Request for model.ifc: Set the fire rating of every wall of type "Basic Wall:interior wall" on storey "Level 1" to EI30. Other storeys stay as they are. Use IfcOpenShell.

First a look at what the model holds.

```python
import ifcopenshell
import ifcopenshell.util.element

model = ifcopenshell.open("model.ifc")
print(model.schema)
storey = next(s for s in model.by_type("IfcBuildingStorey") if s.Name == "Level 1")
walls = [e for e in ifcopenshell.util.element.get_decomposition(storey) if e.is_a("IfcWall")]
seen = {}
for e in walls:
    element_type = ifcopenshell.util.element.get_type(e)
    key = (element_type.Name if element_type != e and element_type else None, ifcopenshell.util.element.get_pset(e, "Pset_WallCommon", "FireRating"))
    seen[key] = seen.get(key, 0) + 1
for (name, value), count in sorted(seen.items(), key=str):
    print(count, "x", name, "|", value)
```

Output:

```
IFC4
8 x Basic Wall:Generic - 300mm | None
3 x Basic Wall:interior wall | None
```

```python
import ifcopenshell
import ifcopenshell.api.pset
import ifcopenshell.util.element

model = ifcopenshell.open("model.ifc")

storey = next(s for s in model.by_type("IfcBuildingStorey") if s.Name == "Level 1")
walls = [e for e in ifcopenshell.util.element.get_decomposition(storey) if e.is_a("IfcWall")]

count = 0
for e in walls:
    element_type = ifcopenshell.util.element.get_type(e)
    if element_type in (None, e) or element_type.Name != "Basic Wall:interior wall":
        continue
    # add_pset returns the element's existing set when there is one.
    pset = ifcopenshell.api.pset.add_pset(model, product=e, name="Pset_WallCommon")
    ifcopenshell.api.pset.edit_pset(model, pset=pset, properties={"FireRating": "EI30"})
    count += 1

print(count, "walls updated")

model.write("model_edited.ifc")
```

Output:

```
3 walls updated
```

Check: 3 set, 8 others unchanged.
